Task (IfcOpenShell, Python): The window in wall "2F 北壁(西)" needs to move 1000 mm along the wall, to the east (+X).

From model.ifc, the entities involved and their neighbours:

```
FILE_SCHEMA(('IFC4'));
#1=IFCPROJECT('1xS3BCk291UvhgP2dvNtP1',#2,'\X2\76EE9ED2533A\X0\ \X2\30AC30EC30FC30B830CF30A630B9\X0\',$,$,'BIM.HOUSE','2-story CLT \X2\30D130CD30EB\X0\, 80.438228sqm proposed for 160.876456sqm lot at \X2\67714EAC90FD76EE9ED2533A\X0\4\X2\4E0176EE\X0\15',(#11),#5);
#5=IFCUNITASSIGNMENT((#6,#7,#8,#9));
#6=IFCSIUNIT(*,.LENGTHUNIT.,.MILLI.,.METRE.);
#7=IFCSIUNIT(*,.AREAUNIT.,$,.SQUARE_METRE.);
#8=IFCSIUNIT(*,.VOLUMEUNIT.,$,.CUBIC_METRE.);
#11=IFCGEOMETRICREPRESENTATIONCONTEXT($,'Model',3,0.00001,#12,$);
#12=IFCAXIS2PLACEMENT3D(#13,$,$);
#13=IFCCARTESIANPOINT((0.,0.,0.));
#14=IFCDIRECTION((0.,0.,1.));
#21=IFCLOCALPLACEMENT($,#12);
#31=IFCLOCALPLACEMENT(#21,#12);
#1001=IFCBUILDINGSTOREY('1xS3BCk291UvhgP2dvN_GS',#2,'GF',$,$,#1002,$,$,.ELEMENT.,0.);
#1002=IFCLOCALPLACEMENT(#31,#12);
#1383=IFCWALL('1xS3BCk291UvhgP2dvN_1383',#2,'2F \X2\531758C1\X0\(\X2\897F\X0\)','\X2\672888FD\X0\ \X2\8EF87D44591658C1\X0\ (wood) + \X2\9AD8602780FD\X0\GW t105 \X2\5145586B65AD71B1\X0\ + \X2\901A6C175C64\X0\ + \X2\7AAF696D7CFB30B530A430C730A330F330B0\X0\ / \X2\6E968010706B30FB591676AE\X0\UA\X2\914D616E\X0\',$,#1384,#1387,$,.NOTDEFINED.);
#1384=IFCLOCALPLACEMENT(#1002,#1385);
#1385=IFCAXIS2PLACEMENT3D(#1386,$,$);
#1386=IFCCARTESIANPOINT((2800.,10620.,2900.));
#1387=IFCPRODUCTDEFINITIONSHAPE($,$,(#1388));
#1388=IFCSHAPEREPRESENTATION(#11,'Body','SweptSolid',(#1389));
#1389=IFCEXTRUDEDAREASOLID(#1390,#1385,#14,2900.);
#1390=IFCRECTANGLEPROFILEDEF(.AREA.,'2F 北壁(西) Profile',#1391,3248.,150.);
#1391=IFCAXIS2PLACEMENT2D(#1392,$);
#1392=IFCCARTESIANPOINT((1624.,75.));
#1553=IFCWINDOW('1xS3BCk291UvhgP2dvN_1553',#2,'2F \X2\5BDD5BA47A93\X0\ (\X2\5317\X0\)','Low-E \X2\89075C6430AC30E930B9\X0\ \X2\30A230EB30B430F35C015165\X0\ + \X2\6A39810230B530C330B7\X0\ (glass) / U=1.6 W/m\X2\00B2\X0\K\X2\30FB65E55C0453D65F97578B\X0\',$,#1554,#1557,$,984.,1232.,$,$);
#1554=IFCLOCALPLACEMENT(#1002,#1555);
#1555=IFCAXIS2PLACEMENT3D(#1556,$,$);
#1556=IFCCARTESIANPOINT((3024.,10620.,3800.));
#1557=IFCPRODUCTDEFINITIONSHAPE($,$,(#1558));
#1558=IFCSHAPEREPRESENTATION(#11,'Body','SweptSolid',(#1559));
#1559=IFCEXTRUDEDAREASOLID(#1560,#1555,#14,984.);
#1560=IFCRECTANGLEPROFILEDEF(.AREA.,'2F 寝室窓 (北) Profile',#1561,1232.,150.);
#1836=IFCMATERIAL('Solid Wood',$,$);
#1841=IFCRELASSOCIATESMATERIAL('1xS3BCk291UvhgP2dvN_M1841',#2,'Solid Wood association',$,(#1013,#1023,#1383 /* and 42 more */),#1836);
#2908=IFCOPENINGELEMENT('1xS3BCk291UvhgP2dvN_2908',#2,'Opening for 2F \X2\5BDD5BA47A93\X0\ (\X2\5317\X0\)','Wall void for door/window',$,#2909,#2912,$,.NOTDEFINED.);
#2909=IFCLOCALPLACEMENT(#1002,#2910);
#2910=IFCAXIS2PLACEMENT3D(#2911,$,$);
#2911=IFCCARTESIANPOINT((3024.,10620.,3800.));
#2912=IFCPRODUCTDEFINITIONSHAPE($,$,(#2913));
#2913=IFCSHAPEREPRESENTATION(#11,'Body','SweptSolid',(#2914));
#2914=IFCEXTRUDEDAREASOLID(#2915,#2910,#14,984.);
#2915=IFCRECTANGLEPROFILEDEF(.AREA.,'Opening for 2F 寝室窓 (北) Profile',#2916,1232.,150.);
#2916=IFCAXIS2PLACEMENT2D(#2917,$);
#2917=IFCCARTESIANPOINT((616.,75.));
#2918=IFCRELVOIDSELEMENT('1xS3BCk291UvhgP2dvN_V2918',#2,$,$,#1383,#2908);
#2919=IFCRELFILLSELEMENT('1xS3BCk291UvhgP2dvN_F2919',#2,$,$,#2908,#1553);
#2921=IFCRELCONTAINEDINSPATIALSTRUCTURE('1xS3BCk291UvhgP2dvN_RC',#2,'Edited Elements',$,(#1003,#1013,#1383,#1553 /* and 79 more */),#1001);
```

```python
import ifcopenshell
import ifcopenshell.api.geometry
import ifcopenshell.util.placement

model = ifcopenshell.open("model.ifc")

window = model.by_guid("1xS3BCk291UvhgP2dvN_1553")
opening = window.FillsVoids[0].RelatingOpeningElement
wall = opening.VoidsElements[0].RelatingBuildingElement

wall_matrix = ifcopenshell.util.placement.get_local_placement(wall.ObjectPlacement)
shift = wall_matrix[:3, 0] * 1000.0
before = ifcopenshell.util.placement.get_local_placement(window.ObjectPlacement)[:3, 3].copy()

# The window is not placed relative to its opening, so move both.
for product in (opening, window):
    matrix = ifcopenshell.util.placement.get_local_placement(product.ObjectPlacement)
    matrix[:3, 3] += shift
    ifcopenshell.api.geometry.edit_object_placement(model, product=product, matrix=matrix, is_si=False)

after = ifcopenshell.util.placement.get_local_placement(window.ObjectPlacement)[:3, 3]
print("window moved by", (after - before).round(3) + 0.0)

model.write("model_updated.ifc")
```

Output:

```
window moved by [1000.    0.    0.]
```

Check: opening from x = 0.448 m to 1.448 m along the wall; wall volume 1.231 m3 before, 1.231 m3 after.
